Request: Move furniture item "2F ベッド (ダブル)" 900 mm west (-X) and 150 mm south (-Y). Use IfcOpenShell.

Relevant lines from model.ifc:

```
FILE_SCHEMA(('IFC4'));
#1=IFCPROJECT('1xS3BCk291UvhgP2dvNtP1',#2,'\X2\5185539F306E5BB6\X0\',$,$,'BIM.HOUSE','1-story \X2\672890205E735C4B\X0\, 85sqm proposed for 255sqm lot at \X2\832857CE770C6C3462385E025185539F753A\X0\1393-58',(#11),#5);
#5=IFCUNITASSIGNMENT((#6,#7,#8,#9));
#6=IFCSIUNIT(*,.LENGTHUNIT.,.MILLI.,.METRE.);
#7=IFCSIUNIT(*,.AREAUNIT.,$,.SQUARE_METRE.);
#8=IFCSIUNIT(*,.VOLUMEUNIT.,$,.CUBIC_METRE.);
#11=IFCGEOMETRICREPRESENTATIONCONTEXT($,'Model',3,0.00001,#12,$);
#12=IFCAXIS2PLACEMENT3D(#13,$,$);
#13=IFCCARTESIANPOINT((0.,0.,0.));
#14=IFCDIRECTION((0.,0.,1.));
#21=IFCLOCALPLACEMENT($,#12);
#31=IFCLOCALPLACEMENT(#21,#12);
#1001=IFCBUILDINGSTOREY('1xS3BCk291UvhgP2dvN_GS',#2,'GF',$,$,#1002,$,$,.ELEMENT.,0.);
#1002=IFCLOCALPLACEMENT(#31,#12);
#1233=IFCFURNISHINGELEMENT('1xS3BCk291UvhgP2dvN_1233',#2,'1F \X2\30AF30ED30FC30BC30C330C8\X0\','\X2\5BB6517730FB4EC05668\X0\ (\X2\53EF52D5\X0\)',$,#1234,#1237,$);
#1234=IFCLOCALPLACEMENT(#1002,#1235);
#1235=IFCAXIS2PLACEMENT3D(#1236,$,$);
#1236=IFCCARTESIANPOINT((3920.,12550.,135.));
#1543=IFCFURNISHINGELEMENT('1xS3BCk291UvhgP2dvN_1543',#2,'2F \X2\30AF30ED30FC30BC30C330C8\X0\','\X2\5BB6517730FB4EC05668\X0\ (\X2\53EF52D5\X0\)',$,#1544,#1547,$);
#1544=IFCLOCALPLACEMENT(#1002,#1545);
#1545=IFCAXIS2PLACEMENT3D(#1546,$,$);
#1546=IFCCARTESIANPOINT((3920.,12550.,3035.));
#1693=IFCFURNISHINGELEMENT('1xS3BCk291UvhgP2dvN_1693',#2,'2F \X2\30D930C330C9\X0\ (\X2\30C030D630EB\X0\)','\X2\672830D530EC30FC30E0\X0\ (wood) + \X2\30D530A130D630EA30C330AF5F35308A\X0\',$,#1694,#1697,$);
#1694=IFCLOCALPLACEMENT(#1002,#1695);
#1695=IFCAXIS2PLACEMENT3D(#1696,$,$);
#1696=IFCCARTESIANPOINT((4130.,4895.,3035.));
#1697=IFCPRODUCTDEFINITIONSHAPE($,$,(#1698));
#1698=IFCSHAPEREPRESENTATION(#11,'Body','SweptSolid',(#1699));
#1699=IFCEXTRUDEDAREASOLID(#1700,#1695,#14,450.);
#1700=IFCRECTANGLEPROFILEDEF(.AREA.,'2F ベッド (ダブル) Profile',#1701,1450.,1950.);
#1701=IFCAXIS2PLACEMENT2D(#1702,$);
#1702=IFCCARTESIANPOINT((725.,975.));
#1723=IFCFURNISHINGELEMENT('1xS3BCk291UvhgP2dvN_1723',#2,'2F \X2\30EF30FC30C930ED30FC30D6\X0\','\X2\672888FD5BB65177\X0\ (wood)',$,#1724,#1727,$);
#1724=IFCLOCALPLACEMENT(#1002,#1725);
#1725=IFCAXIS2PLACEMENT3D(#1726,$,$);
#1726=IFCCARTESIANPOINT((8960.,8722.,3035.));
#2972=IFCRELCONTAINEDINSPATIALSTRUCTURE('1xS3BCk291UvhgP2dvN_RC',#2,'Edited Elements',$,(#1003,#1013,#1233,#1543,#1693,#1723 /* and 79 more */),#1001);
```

```python
import ifcopenshell
import ifcopenshell.api.geometry
import ifcopenshell.util.placement

model = ifcopenshell.open("model.ifc")

item = model.by_guid("1xS3BCk291UvhgP2dvN_1693")
matrix = ifcopenshell.util.placement.get_local_placement(item.ObjectPlacement)
matrix[0, 3] -= 900.0
matrix[1, 3] -= 150.0
ifcopenshell.api.geometry.edit_object_placement(model, product=item, matrix=matrix, is_si=False)

print(ifcopenshell.util.placement.get_local_placement(item.ObjectPlacement).round(3) + 0.0)

model.write("model-out.ifc")
```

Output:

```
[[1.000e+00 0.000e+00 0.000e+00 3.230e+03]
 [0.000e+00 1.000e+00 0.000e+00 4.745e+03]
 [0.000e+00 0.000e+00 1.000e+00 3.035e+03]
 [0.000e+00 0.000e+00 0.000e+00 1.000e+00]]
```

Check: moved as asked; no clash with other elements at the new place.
